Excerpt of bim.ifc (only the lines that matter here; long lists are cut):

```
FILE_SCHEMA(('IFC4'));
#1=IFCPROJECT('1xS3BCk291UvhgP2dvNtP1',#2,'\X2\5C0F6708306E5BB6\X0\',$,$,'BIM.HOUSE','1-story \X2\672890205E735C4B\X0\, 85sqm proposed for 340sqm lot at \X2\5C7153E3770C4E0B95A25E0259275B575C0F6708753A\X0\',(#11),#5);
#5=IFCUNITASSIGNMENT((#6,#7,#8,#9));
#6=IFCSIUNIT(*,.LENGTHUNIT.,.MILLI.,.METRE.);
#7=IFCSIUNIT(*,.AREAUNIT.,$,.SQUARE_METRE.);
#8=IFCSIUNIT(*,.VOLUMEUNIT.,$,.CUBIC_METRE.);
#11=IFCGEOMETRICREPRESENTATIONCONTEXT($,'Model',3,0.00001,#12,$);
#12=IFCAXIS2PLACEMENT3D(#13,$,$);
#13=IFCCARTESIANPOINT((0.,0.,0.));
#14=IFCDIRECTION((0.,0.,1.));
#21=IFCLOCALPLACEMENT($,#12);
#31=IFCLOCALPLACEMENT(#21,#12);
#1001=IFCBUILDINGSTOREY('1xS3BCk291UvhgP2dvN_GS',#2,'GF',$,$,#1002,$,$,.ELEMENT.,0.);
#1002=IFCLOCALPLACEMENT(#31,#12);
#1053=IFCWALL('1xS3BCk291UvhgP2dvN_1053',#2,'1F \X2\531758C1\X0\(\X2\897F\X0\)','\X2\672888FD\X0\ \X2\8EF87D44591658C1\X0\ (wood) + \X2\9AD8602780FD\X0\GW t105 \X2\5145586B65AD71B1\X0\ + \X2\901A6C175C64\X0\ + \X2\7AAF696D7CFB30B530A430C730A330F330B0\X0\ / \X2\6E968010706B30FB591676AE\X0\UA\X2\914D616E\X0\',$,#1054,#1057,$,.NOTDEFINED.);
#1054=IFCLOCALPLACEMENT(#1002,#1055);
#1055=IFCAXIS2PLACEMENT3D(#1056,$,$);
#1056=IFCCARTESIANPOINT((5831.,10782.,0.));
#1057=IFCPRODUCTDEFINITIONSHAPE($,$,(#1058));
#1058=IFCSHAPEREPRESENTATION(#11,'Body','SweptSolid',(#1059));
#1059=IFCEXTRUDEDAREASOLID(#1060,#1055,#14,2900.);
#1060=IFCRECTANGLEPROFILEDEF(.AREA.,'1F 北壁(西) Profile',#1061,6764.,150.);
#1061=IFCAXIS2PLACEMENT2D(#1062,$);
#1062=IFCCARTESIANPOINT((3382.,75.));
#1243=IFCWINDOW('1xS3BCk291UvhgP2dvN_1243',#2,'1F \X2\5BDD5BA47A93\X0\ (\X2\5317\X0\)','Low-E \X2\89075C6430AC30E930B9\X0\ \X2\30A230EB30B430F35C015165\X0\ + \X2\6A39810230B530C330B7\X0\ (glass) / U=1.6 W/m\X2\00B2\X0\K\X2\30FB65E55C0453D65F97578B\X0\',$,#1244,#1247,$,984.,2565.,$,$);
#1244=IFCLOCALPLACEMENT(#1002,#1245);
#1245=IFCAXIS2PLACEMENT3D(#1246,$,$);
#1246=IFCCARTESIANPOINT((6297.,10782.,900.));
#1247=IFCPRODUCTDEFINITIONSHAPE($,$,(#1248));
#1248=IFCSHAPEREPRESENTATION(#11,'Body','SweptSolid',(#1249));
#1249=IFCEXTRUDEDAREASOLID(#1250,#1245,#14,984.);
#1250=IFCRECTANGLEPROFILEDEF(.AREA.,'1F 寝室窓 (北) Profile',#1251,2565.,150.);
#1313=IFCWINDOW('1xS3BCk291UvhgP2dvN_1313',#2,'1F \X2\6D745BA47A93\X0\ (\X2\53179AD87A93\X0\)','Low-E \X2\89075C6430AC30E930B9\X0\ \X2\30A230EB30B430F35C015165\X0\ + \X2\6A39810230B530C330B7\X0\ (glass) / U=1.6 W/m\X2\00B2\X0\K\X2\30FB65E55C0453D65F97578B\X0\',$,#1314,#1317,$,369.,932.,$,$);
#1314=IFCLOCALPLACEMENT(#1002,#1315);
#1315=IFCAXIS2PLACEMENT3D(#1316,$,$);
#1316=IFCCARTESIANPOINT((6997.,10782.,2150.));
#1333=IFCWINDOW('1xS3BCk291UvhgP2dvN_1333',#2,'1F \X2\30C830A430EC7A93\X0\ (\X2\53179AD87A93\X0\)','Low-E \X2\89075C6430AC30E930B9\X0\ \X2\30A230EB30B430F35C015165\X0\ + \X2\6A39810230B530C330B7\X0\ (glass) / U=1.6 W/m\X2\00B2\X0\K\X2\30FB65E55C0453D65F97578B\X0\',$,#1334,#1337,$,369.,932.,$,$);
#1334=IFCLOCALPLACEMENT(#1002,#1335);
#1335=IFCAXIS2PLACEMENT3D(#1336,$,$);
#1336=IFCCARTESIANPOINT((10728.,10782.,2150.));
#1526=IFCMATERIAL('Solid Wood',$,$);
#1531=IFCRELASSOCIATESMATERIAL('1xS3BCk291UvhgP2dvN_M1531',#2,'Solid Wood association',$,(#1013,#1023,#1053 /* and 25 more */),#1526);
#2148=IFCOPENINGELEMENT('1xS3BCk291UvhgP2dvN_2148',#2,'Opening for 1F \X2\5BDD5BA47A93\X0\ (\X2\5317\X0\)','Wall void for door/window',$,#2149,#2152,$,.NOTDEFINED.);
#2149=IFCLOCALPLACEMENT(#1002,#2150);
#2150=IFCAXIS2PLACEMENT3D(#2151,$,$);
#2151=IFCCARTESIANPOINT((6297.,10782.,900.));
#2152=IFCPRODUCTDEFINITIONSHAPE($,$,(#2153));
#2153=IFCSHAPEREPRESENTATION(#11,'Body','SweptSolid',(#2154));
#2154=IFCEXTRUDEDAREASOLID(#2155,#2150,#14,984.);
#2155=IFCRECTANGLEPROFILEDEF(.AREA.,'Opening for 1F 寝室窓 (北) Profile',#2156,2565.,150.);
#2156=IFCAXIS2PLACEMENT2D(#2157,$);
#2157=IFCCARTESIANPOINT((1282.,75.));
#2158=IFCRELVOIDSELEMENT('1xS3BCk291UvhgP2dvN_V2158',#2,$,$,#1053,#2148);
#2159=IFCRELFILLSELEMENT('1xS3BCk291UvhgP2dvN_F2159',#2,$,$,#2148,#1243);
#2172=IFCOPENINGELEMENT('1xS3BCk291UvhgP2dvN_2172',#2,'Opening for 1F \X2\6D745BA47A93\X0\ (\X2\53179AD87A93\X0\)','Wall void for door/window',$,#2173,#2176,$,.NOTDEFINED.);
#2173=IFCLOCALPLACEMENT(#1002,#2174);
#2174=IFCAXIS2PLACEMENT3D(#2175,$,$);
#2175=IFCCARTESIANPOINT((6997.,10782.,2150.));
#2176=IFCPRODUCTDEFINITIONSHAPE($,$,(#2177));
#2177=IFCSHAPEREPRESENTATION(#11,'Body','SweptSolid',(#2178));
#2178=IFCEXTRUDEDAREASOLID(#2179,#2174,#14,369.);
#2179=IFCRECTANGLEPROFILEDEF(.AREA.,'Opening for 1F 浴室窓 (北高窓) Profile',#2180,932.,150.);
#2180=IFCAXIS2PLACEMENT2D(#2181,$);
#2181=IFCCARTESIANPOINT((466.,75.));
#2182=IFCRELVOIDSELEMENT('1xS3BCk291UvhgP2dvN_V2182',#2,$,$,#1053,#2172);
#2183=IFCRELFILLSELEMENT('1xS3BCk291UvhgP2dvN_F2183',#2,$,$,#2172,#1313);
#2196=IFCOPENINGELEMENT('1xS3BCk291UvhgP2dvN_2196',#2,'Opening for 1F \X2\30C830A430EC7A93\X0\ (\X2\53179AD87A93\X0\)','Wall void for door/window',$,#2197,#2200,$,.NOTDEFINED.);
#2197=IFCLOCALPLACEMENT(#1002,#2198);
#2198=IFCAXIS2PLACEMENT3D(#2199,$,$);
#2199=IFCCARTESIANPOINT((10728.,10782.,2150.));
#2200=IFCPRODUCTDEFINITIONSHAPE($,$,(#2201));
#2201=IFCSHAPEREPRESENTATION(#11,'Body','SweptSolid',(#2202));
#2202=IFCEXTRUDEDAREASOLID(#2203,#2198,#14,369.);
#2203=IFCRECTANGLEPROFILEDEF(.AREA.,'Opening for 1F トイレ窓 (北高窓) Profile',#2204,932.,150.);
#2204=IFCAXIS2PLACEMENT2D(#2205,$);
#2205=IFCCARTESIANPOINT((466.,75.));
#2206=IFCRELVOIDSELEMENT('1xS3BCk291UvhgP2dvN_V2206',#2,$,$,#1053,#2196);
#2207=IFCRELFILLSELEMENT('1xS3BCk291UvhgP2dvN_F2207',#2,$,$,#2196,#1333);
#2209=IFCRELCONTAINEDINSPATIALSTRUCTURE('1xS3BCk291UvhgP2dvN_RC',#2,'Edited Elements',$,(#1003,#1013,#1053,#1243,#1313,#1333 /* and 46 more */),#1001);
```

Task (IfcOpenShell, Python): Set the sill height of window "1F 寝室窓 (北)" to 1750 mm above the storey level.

```python
import numpy as np
import ifcopenshell
import ifcopenshell.api.geometry
import ifcopenshell.geom
import ifcopenshell.util.element
import ifcopenshell.util.placement
import ifcopenshell.util.shape
import ifcopenshell.util.unit

model = ifcopenshell.open("bim.ifc")
unit_scale = ifcopenshell.util.unit.calculate_unit_scale(model)

window = model.by_guid("1xS3BCk291UvhgP2dvN_1243")
opening = window.FillsVoids[0].RelatingOpeningElement
storey = ifcopenshell.util.element.get_container(window, ifc_class="IfcBuildingStorey")
level = ifcopenshell.util.placement.get_local_placement(storey.ObjectPlacement)[2, 3]

# The opening's origin need not be at the sill, so measure its lowest point.
shape = ifcopenshell.geom.create_shape(ifcopenshell.geom.settings(), opening)
bottom = ifcopenshell.util.shape.get_shape_bottom_elevation(shape, shape.geometry) / unit_scale
dz = level + 1750.0 - bottom

shift = np.array([0.0, 0.0, dz])
# The window is not placed relative to its opening, so move both.
for product in (opening, window):
    matrix = ifcopenshell.util.placement.get_local_placement(product.ObjectPlacement)
    matrix[:3, 3] += shift
    ifcopenshell.api.geometry.edit_object_placement(model, product=product, matrix=matrix, is_si=False)

print(f"moved by {dz * unit_scale:+.3f} m")

model.write("bim_v2.ifc")
```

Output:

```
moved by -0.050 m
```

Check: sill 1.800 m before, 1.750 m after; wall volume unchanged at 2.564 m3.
